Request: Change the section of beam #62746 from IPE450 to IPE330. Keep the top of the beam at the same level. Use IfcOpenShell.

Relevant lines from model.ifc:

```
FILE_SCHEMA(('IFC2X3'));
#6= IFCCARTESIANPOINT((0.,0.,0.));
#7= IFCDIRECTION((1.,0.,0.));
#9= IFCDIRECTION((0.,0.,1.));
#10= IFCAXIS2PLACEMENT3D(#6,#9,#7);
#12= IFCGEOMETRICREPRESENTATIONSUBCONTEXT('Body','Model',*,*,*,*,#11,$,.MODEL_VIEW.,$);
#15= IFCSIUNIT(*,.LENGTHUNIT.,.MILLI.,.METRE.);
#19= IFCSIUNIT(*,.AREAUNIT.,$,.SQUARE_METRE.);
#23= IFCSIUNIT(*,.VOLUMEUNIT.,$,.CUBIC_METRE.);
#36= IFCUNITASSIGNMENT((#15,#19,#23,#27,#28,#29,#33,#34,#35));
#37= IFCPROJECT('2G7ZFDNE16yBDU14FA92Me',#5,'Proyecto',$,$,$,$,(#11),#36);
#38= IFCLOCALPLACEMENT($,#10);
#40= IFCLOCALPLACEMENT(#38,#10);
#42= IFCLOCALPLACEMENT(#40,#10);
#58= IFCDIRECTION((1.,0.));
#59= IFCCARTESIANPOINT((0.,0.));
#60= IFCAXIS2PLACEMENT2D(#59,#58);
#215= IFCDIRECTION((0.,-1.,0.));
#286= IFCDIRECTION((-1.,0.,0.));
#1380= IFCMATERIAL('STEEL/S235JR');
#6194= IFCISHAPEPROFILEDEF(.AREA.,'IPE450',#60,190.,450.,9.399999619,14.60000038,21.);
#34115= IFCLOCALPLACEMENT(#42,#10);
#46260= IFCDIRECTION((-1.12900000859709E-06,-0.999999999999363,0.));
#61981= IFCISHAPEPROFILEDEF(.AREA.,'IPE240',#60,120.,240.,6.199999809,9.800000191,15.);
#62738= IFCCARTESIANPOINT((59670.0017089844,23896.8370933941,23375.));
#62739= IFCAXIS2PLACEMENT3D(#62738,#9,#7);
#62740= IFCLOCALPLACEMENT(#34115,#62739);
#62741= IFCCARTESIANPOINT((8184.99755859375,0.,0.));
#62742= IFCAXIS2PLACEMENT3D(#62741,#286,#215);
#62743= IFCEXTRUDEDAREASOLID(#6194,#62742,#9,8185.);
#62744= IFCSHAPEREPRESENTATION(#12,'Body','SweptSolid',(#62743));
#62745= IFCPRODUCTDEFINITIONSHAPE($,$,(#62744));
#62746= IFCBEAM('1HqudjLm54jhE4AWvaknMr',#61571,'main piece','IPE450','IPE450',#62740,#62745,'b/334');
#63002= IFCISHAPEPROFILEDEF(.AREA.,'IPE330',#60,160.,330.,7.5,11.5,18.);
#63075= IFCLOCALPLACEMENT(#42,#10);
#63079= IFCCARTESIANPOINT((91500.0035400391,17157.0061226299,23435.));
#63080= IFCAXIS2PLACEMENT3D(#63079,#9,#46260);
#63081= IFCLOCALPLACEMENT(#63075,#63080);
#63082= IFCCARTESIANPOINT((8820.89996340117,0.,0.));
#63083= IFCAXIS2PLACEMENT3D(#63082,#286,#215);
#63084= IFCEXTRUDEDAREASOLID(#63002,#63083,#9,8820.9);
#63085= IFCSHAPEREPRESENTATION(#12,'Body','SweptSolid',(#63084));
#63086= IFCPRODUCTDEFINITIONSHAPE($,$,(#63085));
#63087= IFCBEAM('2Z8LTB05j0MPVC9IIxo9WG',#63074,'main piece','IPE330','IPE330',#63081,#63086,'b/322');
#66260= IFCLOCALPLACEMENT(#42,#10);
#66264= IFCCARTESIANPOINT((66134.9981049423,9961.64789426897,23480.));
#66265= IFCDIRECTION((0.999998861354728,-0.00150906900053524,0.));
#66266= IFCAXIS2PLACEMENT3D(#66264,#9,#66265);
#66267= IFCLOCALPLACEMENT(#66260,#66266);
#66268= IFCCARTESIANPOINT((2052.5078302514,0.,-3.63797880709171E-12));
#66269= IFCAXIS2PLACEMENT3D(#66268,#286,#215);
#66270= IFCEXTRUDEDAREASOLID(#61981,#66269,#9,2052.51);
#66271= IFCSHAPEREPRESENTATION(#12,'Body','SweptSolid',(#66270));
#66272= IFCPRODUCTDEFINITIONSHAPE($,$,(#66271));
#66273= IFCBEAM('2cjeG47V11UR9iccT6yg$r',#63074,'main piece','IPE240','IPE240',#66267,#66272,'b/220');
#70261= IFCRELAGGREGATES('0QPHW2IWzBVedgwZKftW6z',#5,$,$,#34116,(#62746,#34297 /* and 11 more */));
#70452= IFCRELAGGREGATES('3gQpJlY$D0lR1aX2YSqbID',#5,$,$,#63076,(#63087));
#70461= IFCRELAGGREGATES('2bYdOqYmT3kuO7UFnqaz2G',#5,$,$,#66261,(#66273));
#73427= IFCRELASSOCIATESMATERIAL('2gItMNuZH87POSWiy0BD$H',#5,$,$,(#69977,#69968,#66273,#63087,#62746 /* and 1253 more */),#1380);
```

```python
import ifcopenshell
import ifcopenshell.util.element
import ifcopenshell.util.representation

model = ifcopenshell.open("model.ifc")

member = model.by_guid("1HqudjLm54jhE4AWvaknMr")
source = next(p for p in model.by_type("IfcIShapeProfileDef") if p.ProfileName == "IPE330")

body = ifcopenshell.util.representation.get_representation(member, "Model", "Body")
solid = body.Items[0]
old_profile = solid.SweptArea

# Copy the section's sizes but keep this member's own profile position.
profile = ifcopenshell.util.element.copy(model, source)
# Profiles are centred, so shift by half the change in depth to hold the top.
shift = (old_profile.OverallDepth - profile.OverallDepth) / 2
x, y = old_profile.Position.Location.Coordinates
up = (0.0, 1.0)  # upwards, in the solid's own plane
location = model.createIfcCartesianPoint((x + up[0] * shift, y + up[1] * shift))
profile.Position = model.createIfcAxis2Placement2D(location, old_profile.Position.RefDirection)
solid.SweptArea = profile
if not model.get_total_inverses(old_profile):
    ifcopenshell.util.element.remove_deep2(model, old_profile)
member.Description = member.Description.replace("IPE450", "IPE330")
member.ObjectType = member.ObjectType.replace("IPE450", "IPE330")

print(solid.SweptArea)

model.write("model_edited.ifc")
```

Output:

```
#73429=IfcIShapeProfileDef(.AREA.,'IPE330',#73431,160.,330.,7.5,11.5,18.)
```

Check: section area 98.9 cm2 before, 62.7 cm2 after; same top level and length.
